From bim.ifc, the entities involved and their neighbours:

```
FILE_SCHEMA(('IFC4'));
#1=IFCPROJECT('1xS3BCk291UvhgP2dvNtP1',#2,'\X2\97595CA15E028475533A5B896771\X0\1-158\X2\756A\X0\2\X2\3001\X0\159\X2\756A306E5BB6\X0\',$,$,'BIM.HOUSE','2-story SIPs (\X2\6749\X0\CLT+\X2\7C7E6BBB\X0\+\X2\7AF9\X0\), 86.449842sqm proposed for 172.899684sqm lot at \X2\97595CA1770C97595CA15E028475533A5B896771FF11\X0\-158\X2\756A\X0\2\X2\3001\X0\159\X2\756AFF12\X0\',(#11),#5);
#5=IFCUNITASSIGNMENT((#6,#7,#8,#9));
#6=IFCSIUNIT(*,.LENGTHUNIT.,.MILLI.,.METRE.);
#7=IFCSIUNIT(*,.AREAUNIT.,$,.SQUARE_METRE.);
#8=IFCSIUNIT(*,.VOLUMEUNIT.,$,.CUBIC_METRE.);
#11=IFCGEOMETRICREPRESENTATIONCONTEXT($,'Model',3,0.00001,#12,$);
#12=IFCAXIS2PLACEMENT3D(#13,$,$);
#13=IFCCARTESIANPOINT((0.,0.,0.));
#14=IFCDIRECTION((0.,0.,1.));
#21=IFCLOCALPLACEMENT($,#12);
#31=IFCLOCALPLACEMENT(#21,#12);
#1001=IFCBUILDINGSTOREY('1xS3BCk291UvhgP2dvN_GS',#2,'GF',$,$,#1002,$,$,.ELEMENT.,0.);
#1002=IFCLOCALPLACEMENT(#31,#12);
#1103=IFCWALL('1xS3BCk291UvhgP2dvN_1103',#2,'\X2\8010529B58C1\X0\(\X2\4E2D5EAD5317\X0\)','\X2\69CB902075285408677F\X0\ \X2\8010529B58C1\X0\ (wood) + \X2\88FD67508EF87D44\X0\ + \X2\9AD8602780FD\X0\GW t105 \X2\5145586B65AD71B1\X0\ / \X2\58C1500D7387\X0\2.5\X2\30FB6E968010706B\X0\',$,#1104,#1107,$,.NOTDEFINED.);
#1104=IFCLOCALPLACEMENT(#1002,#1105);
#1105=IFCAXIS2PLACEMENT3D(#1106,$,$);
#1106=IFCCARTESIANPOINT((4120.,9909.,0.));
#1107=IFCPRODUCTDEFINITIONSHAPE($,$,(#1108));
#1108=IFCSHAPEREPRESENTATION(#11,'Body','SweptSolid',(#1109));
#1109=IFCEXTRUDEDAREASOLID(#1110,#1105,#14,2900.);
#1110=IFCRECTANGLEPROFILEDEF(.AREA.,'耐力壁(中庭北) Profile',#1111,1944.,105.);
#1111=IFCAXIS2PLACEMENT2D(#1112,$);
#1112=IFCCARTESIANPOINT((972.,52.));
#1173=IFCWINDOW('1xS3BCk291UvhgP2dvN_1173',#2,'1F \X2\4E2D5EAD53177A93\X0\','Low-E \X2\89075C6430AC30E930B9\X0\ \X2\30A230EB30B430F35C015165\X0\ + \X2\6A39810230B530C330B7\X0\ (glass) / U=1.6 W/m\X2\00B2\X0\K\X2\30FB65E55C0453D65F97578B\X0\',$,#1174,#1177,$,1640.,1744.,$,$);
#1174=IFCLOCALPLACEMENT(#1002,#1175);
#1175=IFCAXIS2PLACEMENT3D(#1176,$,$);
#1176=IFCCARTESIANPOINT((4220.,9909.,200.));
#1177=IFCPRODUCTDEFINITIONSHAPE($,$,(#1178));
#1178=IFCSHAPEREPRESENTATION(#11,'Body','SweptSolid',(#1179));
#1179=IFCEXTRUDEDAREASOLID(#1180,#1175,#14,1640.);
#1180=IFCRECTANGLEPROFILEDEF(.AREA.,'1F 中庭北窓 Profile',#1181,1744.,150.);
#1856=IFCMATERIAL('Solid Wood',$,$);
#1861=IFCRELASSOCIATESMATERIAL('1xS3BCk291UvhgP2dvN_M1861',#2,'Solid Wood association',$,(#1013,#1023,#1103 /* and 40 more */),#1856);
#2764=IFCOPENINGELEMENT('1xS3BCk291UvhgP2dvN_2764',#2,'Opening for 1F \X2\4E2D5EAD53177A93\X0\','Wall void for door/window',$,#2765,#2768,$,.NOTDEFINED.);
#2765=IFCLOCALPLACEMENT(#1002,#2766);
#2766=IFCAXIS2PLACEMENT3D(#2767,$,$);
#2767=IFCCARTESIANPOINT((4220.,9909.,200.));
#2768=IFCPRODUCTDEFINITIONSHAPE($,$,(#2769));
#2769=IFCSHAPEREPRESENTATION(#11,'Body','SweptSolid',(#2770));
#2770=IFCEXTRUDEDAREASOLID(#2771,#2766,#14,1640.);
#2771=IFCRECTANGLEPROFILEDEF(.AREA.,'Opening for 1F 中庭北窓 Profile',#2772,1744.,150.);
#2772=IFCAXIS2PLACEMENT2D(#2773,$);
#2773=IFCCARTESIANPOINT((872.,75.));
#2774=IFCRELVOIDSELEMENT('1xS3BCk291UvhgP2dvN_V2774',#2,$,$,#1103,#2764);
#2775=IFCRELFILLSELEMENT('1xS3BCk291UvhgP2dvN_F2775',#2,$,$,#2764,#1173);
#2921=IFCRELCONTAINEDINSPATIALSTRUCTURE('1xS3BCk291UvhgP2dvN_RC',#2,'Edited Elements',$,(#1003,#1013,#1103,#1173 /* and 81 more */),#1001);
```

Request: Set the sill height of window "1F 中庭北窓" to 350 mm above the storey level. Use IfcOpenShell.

```python
import numpy as np
import ifcopenshell
import ifcopenshell.api.geometry
import ifcopenshell.geom
import ifcopenshell.util.element
import ifcopenshell.util.placement
import ifcopenshell.util.shape
import ifcopenshell.util.unit

model = ifcopenshell.open("bim.ifc")
unit_scale = ifcopenshell.util.unit.calculate_unit_scale(model)

window = model.by_id(1173)
opening = window.FillsVoids[0].RelatingOpeningElement
storey = ifcopenshell.util.element.get_container(window, ifc_class="IfcBuildingStorey")
level = ifcopenshell.util.placement.get_local_placement(storey.ObjectPlacement)[2, 3]

# The opening's origin need not be at the sill, so measure its lowest point.
shape = ifcopenshell.geom.create_shape(ifcopenshell.geom.settings(), opening)
bottom = ifcopenshell.util.shape.get_shape_bottom_elevation(shape, shape.geometry) / unit_scale
dz = level + 0.35 / unit_scale - bottom

shift = np.array([0.0, 0.0, dz])
# The window is not placed relative to its opening, so move both.
for product in (opening, window):
    matrix = ifcopenshell.util.placement.get_local_placement(product.ObjectPlacement)
    matrix[:3, 3] += shift
    ifcopenshell.api.geometry.edit_object_placement(model, product=product, matrix=matrix, is_si=False)

print(f"moved by {dz * unit_scale:+.3f} m")

model.write("bim_v2.ifc")
```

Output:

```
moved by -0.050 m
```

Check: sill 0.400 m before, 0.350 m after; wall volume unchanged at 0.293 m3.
